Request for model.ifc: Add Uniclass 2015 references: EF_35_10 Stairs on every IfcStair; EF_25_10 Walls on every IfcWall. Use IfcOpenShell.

First a look at what the model holds.

```python
import ifcopenshell

model = ifcopenshell.open("model.ifc")
print(model.schema)
print("classifications:", [c.Name for c in model.by_type("IfcClassification")])
for ifc_class in ("IfcDoor", "IfcRoof", "IfcStair", "IfcWall", "IfcWindow"):
    print(ifc_class, len(model.by_type(ifc_class)))
```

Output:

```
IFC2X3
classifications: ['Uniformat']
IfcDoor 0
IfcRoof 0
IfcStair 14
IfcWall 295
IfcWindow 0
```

```python
import ifcopenshell
import ifcopenshell.api.classification

model = ifcopenshell.open("model.ifc")

# IFC2X3 requires Source and Edition and has no link from the project to the system.
system = model.create_entity("IfcClassification", Source="NBS", Edition="2015", Name="Uniclass 2015")

codes = {
    "IfcStair": ("EF_35_10", "Stairs"),
    "IfcWall": ("EF_25_10", "Walls"),
}
for ifc_class, (code, name) in codes.items():
    products = model.by_type(ifc_class)
    ifcopenshell.api.classification.add_reference(
        model, products=products, classification=system, identification=code, name=name
    )
    print(code, len(products))

model.write("model-out.ifc")
```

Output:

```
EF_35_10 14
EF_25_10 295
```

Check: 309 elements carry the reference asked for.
